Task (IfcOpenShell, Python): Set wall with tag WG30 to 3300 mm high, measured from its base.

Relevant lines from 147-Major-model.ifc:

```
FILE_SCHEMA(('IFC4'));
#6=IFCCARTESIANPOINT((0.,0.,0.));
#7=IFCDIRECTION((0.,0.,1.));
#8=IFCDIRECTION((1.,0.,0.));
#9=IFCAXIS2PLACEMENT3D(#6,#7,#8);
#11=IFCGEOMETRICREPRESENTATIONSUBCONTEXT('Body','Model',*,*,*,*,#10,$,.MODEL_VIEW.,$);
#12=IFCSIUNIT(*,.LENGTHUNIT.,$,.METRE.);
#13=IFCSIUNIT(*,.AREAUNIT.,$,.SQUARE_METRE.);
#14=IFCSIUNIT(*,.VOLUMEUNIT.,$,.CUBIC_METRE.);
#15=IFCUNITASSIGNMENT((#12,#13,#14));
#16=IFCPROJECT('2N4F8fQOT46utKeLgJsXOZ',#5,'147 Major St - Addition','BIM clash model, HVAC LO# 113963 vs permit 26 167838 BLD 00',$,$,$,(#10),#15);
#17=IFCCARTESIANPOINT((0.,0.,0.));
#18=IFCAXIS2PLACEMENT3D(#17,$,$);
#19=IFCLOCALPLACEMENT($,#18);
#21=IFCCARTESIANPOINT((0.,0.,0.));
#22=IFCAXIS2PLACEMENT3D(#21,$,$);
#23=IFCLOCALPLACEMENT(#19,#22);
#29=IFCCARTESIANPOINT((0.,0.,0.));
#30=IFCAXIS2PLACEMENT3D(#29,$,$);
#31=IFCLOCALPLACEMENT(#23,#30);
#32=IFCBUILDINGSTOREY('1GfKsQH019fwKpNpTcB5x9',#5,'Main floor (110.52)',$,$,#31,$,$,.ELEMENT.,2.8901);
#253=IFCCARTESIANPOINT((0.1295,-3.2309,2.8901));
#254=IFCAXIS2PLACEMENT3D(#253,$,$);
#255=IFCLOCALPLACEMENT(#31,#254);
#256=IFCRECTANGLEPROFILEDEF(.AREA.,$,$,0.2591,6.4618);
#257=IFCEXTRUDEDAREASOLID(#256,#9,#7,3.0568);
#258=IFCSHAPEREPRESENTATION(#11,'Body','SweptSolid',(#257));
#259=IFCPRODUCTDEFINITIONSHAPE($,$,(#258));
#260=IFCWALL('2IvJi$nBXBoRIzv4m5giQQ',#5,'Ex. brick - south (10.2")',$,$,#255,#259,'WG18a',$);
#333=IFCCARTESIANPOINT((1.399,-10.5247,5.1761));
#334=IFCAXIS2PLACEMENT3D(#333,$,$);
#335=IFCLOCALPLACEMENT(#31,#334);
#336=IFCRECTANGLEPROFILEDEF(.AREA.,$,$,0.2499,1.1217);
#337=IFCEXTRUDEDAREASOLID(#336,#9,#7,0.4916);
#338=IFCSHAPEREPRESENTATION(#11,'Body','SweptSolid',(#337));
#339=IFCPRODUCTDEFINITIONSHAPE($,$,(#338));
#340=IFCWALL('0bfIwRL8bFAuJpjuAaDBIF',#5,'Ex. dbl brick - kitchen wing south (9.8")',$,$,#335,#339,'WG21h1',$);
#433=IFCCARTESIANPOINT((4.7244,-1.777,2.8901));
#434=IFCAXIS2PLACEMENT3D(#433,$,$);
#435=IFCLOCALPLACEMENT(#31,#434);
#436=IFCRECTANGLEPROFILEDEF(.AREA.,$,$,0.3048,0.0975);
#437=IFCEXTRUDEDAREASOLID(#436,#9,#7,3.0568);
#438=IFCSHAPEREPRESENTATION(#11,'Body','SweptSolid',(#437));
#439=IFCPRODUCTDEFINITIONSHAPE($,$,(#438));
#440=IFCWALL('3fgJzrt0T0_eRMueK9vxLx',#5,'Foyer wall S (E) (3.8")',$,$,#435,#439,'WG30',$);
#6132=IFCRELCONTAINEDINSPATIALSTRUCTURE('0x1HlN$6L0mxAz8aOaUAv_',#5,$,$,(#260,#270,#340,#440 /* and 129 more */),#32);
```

```python
import ifcopenshell
import ifcopenshell.geom
import ifcopenshell.util.representation
import ifcopenshell.util.shape
import ifcopenshell.util.unit

model = ifcopenshell.open("147-Major-model.ifc")
unit_scale = ifcopenshell.util.unit.calculate_unit_scale(model)
settings = ifcopenshell.geom.settings()


def volume(element):
    """Net volume in cubic metres, openings subtracted."""
    shape = ifcopenshell.geom.create_shape(settings, element)
    return ifcopenshell.util.shape.get_volume(shape.geometry)


wall = model.by_guid("3fgJzrt0T0_eRMueK9vxLx")
before = volume(wall)

body = ifcopenshell.util.representation.get_representation(wall, "Model", "Body")
solid = body.Items[0]
old_height = solid.Depth
solid.Depth = 3.3 / unit_scale
after = volume(wall)

print(f"height {old_height:g} -> {solid.Depth:g}, volume {before:.3f} -> {after:.3f} m3")

model.write("147-Major-model_v2.ifc")
```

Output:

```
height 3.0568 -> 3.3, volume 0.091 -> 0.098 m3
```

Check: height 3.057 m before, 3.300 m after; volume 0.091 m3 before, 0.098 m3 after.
